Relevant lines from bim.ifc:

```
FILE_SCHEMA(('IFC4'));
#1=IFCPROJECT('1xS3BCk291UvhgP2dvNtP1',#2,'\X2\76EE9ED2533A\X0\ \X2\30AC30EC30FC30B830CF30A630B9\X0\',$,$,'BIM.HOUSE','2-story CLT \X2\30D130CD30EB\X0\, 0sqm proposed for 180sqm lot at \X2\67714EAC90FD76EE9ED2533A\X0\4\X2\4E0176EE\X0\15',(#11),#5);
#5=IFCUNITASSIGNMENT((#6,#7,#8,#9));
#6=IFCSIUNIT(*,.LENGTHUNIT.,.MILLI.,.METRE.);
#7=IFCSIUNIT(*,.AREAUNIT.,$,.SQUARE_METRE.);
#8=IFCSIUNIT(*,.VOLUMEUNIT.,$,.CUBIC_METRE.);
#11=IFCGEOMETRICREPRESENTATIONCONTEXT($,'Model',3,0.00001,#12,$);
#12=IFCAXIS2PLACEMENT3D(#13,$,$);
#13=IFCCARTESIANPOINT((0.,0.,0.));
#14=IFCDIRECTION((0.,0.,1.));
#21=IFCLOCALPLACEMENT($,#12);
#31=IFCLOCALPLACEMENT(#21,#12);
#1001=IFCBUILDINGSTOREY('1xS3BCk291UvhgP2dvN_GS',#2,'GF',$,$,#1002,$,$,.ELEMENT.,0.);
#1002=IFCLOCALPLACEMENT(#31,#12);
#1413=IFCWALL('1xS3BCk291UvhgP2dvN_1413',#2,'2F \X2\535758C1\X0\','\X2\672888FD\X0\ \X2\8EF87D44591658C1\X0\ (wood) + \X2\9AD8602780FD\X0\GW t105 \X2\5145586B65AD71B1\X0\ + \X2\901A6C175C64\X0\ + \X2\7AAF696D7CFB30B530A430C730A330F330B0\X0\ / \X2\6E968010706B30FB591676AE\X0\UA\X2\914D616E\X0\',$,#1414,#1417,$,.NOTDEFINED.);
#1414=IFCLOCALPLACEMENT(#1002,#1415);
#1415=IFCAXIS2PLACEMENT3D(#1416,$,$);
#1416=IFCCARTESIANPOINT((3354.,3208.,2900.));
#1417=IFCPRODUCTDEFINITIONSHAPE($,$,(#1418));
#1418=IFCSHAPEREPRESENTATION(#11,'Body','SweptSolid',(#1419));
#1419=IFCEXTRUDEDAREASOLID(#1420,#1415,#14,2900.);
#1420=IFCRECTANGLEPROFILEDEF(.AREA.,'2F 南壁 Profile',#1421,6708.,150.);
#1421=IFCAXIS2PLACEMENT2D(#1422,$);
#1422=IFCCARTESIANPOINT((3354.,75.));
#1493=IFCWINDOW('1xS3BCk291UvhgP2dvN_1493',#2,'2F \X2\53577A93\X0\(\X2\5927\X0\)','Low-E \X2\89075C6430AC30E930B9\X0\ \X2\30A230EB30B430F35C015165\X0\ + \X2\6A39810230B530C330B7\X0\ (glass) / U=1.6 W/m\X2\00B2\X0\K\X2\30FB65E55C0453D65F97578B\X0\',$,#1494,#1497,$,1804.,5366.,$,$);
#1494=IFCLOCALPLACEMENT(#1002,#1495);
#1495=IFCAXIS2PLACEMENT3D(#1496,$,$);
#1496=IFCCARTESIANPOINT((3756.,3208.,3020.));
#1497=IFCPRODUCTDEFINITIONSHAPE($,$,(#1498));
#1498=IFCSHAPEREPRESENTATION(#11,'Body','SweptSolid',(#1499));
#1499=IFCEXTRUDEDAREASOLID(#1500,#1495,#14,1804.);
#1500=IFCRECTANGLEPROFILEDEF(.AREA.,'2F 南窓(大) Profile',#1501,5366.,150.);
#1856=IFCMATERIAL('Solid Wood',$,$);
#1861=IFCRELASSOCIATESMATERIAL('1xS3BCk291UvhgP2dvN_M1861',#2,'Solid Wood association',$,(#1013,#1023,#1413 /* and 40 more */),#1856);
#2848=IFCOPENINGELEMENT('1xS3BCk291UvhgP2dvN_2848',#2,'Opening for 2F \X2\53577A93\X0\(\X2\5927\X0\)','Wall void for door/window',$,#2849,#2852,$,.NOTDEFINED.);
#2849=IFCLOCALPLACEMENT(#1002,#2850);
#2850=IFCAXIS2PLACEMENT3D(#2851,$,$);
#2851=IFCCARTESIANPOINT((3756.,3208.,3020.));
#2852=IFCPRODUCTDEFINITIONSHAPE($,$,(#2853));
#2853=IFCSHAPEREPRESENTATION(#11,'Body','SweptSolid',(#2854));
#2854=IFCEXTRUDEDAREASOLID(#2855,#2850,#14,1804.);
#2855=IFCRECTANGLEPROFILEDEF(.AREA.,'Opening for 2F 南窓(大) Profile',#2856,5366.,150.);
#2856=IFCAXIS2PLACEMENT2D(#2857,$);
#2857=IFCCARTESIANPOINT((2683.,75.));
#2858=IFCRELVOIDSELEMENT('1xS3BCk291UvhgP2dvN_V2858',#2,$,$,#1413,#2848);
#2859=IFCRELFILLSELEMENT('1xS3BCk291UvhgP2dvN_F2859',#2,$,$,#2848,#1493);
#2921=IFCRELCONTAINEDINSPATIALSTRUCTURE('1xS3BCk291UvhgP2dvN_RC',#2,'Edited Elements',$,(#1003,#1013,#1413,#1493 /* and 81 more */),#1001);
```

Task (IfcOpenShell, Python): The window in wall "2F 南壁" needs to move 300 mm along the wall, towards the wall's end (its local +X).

```python
import ifcopenshell
import ifcopenshell.api.geometry
import ifcopenshell.util.placement
import ifcopenshell.util.unit

model = ifcopenshell.open("bim.ifc")
unit_scale = ifcopenshell.util.unit.calculate_unit_scale(model)

window = model.by_guid("1xS3BCk291UvhgP2dvN_1493")
opening = window.FillsVoids[0].RelatingOpeningElement
wall = opening.VoidsElements[0].RelatingBuildingElement

wall_matrix = ifcopenshell.util.placement.get_local_placement(wall.ObjectPlacement)
shift = wall_matrix[:3, 0] * 0.3 / unit_scale
before = ifcopenshell.util.placement.get_local_placement(window.ObjectPlacement)[:3, 3].copy()

# The window is not placed relative to its opening, so move both.
for product in (opening, window):
    matrix = ifcopenshell.util.placement.get_local_placement(product.ObjectPlacement)
    matrix[:3, 3] += shift
    ifcopenshell.api.geometry.edit_object_placement(model, product=product, matrix=matrix, is_si=False)

after = ifcopenshell.util.placement.get_local_placement(window.ObjectPlacement)[:3, 3]
print("window moved by", (after - before).round(3) + 0.0)

model.write("bim_edited.ifc")
```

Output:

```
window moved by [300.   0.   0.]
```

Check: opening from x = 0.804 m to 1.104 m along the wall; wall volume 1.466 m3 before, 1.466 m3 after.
